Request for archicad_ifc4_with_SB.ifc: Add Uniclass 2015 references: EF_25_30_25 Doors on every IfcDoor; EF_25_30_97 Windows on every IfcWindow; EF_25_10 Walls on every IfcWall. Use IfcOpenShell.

First a look at what the model holds.

```python
import ifcopenshell

model = ifcopenshell.open("archicad_ifc4_with_SB.ifc")
print(model.schema)
print("classifications:", [c.Name for c in model.by_type("IfcClassification")])
for ifc_class in ("IfcDoor", "IfcRoof", "IfcStair", "IfcWall", "IfcWindow"):
    print(ifc_class, len(model.by_type(ifc_class)))
```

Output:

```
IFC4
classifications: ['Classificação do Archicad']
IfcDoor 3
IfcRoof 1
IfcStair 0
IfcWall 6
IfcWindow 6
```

```python
import ifcopenshell
import ifcopenshell.api.classification

model = ifcopenshell.open("archicad_ifc4_with_SB.ifc")

system = ifcopenshell.api.classification.add_classification(model, classification="Uniclass 2015")

codes = {
    "IfcDoor": ("EF_25_30_25", "Doors"),
    "IfcWindow": ("EF_25_30_97", "Windows"),
    "IfcWall": ("EF_25_10", "Walls"),
}
for ifc_class, (code, name) in codes.items():
    products = model.by_type(ifc_class)
    ifcopenshell.api.classification.add_reference(
        model, products=products, classification=system, identification=code, name=name
    )
    print(code, len(products))

model.write("archicad_ifc4_with_SB_updated.ifc")
```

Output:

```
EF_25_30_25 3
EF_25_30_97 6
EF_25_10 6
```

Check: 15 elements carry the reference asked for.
